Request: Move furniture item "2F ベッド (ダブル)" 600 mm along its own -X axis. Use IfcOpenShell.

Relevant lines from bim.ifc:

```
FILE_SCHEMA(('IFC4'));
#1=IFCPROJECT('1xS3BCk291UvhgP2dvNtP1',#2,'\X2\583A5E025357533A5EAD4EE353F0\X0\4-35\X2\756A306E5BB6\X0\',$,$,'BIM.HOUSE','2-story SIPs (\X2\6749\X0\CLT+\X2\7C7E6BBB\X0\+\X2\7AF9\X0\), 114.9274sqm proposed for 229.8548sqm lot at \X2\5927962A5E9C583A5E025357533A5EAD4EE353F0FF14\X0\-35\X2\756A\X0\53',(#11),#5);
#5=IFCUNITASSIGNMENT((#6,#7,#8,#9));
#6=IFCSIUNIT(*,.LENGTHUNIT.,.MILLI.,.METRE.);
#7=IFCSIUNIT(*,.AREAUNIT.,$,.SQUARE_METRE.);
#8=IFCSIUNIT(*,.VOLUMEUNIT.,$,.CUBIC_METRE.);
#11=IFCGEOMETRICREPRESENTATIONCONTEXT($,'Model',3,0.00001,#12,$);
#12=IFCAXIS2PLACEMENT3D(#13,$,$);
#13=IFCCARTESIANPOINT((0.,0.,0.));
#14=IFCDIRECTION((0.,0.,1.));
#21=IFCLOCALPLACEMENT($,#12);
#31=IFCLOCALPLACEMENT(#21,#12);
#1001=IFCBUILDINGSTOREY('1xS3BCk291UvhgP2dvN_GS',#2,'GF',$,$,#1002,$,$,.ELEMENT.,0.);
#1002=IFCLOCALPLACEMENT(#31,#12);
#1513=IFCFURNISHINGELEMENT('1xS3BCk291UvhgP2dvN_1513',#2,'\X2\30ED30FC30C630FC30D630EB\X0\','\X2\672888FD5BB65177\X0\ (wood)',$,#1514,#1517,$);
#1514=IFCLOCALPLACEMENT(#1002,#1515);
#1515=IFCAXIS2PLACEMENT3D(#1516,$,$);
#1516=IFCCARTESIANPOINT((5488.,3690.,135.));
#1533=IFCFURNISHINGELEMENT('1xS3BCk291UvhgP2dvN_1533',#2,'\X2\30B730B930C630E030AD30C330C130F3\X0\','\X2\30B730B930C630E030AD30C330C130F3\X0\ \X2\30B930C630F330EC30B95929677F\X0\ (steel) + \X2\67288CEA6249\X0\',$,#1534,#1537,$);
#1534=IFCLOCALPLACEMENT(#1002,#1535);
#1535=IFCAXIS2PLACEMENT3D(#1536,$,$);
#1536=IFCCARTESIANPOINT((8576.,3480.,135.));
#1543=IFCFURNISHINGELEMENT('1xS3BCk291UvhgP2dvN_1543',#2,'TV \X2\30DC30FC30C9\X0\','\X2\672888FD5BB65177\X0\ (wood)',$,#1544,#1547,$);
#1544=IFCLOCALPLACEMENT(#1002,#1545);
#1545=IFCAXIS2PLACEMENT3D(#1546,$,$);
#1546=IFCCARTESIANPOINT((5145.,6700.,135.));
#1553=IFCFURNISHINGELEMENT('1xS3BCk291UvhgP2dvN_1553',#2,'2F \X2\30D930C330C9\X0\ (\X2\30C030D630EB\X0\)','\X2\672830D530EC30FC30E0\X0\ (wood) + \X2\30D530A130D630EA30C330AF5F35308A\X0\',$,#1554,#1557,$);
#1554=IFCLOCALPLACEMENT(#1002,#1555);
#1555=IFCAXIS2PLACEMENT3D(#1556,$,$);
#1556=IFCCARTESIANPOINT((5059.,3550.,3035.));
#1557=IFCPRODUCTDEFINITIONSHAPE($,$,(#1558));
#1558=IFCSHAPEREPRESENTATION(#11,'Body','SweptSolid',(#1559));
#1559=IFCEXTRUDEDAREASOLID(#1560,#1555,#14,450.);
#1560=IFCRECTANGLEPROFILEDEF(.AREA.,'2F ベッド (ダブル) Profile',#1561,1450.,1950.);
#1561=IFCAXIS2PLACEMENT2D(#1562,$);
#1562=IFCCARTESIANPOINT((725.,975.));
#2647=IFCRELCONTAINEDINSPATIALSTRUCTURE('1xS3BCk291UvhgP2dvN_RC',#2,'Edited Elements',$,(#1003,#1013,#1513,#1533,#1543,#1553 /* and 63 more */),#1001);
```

```python
import ifcopenshell
import ifcopenshell.api.geometry
import ifcopenshell.util.placement
import ifcopenshell.util.unit

model = ifcopenshell.open("bim.ifc")
unit_scale = ifcopenshell.util.unit.calculate_unit_scale(model)

item = model.by_guid("1xS3BCk291UvhgP2dvN_1553")
matrix = ifcopenshell.util.placement.get_local_placement(item.ObjectPlacement)
matrix[:3, 3] -= matrix[:3, 0] * 0.6 / unit_scale
ifcopenshell.api.geometry.edit_object_placement(model, product=item, matrix=matrix, is_si=False)

print(ifcopenshell.util.placement.get_local_placement(item.ObjectPlacement).round(3) + 0.0)

model.write("bim-out.ifc")
```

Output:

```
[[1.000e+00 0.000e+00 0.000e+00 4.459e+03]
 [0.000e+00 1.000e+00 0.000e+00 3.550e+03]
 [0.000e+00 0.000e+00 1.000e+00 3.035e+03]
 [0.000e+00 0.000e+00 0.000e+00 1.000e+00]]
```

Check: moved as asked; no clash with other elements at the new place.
